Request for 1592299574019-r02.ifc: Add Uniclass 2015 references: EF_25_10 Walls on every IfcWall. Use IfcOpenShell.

First a look at what the model holds.

```python
import ifcopenshell

model = ifcopenshell.open("1592299574019-r02.ifc")
print(model.schema)
print("classifications:", [c.Name for c in model.by_type("IfcClassification")])
for ifc_class in ("IfcDoor", "IfcRoof", "IfcStair", "IfcWall", "IfcWindow"):
    print(ifc_class, len(model.by_type(ifc_class)))
```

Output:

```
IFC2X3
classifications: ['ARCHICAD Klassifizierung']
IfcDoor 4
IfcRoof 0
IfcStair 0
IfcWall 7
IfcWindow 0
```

```python
import ifcopenshell
import ifcopenshell.api.classification

model = ifcopenshell.open("1592299574019-r02.ifc")

# IFC2X3 requires Source and Edition and has no link from the project to the system.
system = model.create_entity("IfcClassification", Source="NBS", Edition="2015", Name="Uniclass 2015")

codes = {
    "IfcWall": ("EF_25_10", "Walls"),
}
for ifc_class, (code, name) in codes.items():
    products = model.by_type(ifc_class)
    ifcopenshell.api.classification.add_reference(
        model, products=products, classification=system, identification=code, name=name
    )
    print(code, len(products))

model.write("1592299574019-r02_v2.ifc")
```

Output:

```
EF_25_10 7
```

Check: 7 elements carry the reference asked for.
